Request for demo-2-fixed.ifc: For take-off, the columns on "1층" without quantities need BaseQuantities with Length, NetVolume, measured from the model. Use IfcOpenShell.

First a look at what the model holds.

```python
import ifcopenshell
import ifcopenshell.util.element
import ifcopenshell.util.unit

model = ifcopenshell.open("demo-2-fixed.ifc")
print(model.schema)
for unit_type in ("LENGTHUNIT", "AREAUNIT", "VOLUMEUNIT"):
    print(unit_type, ifcopenshell.util.unit.calculate_unit_scale(model, unit_type))
storey = next(s for s in model.by_type("IfcBuildingStorey") if s.Name == "1층")
columns = [e for e in ifcopenshell.util.element.get_decomposition(storey) if e.is_a("IfcColumn")]
for e in sorted(columns, key=lambda e: e.id()):
    print(e.id(), e.is_a(), e.Name, list(ifcopenshell.util.element.get_psets(e, qtos_only=True)), sep=" | ")
```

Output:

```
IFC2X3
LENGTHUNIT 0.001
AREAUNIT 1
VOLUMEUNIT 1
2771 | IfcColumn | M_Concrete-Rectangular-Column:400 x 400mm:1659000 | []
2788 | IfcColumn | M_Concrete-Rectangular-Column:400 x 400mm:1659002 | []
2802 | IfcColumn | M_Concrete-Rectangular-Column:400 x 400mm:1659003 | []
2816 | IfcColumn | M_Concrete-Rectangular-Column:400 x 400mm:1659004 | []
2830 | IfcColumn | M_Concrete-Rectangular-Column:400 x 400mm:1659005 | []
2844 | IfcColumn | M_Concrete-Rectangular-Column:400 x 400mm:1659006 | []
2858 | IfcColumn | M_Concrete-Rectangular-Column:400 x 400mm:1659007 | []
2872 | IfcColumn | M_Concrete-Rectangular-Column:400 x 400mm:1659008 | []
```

```python
import ifcopenshell
import ifcopenshell.api.pset
import ifcopenshell.geom
import ifcopenshell.util.element
import ifcopenshell.util.shape
import ifcopenshell.util.unit

model = ifcopenshell.open("demo-2-fixed.ifc")
unit_scale = ifcopenshell.util.unit.calculate_unit_scale(model)
volume_scale = ifcopenshell.util.unit.calculate_unit_scale(model, "VOLUMEUNIT")
settings = ifcopenshell.geom.settings()

storey = next(s for s in model.by_type("IfcBuildingStorey") if s.Name == "1층")
columns = [e for e in ifcopenshell.util.element.get_decomposition(storey) if e.is_a("IfcColumn")]

for e in sorted(columns, key=lambda e: e.id()):
    if ifcopenshell.util.element.get_psets(e, qtos_only=True, should_inherit=False):
        continue
    # Geometry comes back in metres, in the element's own axes.
    shape = ifcopenshell.geom.create_shape(settings, e)
    values = {
        "Length": ifcopenshell.util.shape.get_z(shape.geometry) / unit_scale,
        "NetVolume": ifcopenshell.util.shape.get_volume(shape.geometry) / volume_scale,
    }
    qto = ifcopenshell.api.pset.add_qto(model, product=e, name="BaseQuantities")
    ifcopenshell.api.pset.edit_qto(model, qto=qto, properties=values)
    print(e.id(), {k: round(v, 3) for k, v in values.items()})

model.write("demo-2-fixed-out.ifc")
```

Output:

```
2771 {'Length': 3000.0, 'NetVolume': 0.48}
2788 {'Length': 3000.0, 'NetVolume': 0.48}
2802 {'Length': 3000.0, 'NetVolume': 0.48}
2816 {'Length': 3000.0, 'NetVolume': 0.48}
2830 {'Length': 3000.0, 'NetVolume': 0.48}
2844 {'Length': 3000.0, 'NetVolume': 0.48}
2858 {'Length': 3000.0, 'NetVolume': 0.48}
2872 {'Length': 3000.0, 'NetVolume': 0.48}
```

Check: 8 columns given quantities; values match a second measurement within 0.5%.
